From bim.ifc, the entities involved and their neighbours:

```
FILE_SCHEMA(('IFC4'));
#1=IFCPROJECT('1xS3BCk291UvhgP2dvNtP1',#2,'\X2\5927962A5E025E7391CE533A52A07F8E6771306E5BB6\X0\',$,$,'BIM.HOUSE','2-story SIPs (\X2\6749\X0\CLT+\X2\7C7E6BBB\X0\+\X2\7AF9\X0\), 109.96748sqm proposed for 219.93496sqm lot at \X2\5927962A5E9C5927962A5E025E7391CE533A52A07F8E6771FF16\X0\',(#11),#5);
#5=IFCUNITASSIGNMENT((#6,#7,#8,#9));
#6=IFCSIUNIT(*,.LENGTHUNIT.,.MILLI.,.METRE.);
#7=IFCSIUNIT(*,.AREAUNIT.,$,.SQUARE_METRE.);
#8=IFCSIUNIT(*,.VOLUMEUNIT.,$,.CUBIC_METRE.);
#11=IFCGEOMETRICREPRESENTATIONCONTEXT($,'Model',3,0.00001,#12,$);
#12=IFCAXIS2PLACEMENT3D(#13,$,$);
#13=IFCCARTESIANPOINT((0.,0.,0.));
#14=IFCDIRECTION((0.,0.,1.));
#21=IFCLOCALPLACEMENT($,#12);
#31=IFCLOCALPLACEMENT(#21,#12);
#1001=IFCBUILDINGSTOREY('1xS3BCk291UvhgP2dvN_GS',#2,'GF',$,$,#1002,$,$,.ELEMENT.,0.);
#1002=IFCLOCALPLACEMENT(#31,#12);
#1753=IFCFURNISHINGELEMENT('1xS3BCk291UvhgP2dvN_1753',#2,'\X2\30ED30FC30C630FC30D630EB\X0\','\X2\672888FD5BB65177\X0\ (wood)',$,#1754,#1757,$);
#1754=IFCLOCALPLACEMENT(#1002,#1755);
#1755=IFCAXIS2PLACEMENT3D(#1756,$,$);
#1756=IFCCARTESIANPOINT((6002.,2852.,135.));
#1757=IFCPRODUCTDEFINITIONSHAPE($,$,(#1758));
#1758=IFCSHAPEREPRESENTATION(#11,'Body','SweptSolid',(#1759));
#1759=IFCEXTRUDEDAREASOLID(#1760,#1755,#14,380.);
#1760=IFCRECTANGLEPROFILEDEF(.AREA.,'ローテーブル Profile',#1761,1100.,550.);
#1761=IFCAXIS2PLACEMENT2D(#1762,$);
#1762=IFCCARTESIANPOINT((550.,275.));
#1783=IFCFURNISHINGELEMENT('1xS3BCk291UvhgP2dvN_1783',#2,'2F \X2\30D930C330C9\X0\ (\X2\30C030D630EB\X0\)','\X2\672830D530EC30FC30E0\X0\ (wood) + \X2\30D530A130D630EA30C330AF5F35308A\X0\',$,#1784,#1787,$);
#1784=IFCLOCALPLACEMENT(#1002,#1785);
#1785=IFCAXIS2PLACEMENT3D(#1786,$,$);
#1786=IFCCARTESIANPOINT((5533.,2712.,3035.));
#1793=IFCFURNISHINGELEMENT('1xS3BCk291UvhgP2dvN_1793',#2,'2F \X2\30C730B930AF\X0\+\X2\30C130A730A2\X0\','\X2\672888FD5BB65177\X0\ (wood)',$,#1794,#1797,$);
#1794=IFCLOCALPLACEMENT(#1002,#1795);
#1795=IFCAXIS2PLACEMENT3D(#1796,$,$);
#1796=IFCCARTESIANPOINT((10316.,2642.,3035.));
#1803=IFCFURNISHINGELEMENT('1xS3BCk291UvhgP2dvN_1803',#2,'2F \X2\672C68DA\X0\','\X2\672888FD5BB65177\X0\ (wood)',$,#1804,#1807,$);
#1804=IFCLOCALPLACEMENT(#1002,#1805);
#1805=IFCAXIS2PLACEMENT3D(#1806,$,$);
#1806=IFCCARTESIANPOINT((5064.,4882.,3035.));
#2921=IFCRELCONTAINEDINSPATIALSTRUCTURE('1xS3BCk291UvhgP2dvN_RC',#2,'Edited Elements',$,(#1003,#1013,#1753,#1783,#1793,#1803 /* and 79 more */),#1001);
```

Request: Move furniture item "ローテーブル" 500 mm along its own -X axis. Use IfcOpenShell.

```python
import ifcopenshell
import ifcopenshell.api.geometry
import ifcopenshell.util.placement
import ifcopenshell.util.unit

model = ifcopenshell.open("bim.ifc")
unit_scale = ifcopenshell.util.unit.calculate_unit_scale(model)

item = model.by_id(1753)
matrix = ifcopenshell.util.placement.get_local_placement(item.ObjectPlacement)
matrix[:3, 3] -= matrix[:3, 0] * 0.5 / unit_scale
ifcopenshell.api.geometry.edit_object_placement(model, product=item, matrix=matrix, is_si=False)

print(ifcopenshell.util.placement.get_local_placement(item.ObjectPlacement).round(3) + 0.0)

model.write("bim_rev.ifc")
```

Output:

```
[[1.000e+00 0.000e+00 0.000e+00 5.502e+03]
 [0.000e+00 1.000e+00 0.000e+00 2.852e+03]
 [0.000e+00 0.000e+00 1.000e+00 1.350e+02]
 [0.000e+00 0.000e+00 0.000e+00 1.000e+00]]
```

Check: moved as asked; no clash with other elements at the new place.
